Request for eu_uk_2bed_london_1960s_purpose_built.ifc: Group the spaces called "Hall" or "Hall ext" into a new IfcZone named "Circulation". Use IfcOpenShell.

First a look at what the model holds.

```python
import ifcopenshell

model = ifcopenshell.open("eu_uk_2bed_london_1960s_purpose_built.ifc")
print(model.schema)
seen = {}
for space in model.by_type("IfcSpace"):
    seen[space.LongName] = seen.get(space.LongName, 0) + 1
for name, count in sorted(seen.items(), key=str):
    print(count, "x", name)
print("zones:", [z.Name for z in model.by_type("IfcZone")][:20])
```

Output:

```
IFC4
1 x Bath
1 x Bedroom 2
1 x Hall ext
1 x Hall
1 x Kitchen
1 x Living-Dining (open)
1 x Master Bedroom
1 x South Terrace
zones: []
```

```python
import ifcopenshell
import ifcopenshell.api.group
import ifcopenshell.api.root

model = ifcopenshell.open("eu_uk_2bed_london_1960s_purpose_built.ifc")

names = {"Hall", "Hall ext"}
spaces = [s for s in model.by_type("IfcSpace") if s.LongName in names]

zone = ifcopenshell.api.root.create_entity(model, ifc_class="IfcZone", name="Circulation")
ifcopenshell.api.group.assign_group(model, products=spaces, group=zone)
print(len(spaces), "spaces in", zone.Name)

model.write("eu_uk_2bed_london_1960s_purpose_built_edited.ifc")
```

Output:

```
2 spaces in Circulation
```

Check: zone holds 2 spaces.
